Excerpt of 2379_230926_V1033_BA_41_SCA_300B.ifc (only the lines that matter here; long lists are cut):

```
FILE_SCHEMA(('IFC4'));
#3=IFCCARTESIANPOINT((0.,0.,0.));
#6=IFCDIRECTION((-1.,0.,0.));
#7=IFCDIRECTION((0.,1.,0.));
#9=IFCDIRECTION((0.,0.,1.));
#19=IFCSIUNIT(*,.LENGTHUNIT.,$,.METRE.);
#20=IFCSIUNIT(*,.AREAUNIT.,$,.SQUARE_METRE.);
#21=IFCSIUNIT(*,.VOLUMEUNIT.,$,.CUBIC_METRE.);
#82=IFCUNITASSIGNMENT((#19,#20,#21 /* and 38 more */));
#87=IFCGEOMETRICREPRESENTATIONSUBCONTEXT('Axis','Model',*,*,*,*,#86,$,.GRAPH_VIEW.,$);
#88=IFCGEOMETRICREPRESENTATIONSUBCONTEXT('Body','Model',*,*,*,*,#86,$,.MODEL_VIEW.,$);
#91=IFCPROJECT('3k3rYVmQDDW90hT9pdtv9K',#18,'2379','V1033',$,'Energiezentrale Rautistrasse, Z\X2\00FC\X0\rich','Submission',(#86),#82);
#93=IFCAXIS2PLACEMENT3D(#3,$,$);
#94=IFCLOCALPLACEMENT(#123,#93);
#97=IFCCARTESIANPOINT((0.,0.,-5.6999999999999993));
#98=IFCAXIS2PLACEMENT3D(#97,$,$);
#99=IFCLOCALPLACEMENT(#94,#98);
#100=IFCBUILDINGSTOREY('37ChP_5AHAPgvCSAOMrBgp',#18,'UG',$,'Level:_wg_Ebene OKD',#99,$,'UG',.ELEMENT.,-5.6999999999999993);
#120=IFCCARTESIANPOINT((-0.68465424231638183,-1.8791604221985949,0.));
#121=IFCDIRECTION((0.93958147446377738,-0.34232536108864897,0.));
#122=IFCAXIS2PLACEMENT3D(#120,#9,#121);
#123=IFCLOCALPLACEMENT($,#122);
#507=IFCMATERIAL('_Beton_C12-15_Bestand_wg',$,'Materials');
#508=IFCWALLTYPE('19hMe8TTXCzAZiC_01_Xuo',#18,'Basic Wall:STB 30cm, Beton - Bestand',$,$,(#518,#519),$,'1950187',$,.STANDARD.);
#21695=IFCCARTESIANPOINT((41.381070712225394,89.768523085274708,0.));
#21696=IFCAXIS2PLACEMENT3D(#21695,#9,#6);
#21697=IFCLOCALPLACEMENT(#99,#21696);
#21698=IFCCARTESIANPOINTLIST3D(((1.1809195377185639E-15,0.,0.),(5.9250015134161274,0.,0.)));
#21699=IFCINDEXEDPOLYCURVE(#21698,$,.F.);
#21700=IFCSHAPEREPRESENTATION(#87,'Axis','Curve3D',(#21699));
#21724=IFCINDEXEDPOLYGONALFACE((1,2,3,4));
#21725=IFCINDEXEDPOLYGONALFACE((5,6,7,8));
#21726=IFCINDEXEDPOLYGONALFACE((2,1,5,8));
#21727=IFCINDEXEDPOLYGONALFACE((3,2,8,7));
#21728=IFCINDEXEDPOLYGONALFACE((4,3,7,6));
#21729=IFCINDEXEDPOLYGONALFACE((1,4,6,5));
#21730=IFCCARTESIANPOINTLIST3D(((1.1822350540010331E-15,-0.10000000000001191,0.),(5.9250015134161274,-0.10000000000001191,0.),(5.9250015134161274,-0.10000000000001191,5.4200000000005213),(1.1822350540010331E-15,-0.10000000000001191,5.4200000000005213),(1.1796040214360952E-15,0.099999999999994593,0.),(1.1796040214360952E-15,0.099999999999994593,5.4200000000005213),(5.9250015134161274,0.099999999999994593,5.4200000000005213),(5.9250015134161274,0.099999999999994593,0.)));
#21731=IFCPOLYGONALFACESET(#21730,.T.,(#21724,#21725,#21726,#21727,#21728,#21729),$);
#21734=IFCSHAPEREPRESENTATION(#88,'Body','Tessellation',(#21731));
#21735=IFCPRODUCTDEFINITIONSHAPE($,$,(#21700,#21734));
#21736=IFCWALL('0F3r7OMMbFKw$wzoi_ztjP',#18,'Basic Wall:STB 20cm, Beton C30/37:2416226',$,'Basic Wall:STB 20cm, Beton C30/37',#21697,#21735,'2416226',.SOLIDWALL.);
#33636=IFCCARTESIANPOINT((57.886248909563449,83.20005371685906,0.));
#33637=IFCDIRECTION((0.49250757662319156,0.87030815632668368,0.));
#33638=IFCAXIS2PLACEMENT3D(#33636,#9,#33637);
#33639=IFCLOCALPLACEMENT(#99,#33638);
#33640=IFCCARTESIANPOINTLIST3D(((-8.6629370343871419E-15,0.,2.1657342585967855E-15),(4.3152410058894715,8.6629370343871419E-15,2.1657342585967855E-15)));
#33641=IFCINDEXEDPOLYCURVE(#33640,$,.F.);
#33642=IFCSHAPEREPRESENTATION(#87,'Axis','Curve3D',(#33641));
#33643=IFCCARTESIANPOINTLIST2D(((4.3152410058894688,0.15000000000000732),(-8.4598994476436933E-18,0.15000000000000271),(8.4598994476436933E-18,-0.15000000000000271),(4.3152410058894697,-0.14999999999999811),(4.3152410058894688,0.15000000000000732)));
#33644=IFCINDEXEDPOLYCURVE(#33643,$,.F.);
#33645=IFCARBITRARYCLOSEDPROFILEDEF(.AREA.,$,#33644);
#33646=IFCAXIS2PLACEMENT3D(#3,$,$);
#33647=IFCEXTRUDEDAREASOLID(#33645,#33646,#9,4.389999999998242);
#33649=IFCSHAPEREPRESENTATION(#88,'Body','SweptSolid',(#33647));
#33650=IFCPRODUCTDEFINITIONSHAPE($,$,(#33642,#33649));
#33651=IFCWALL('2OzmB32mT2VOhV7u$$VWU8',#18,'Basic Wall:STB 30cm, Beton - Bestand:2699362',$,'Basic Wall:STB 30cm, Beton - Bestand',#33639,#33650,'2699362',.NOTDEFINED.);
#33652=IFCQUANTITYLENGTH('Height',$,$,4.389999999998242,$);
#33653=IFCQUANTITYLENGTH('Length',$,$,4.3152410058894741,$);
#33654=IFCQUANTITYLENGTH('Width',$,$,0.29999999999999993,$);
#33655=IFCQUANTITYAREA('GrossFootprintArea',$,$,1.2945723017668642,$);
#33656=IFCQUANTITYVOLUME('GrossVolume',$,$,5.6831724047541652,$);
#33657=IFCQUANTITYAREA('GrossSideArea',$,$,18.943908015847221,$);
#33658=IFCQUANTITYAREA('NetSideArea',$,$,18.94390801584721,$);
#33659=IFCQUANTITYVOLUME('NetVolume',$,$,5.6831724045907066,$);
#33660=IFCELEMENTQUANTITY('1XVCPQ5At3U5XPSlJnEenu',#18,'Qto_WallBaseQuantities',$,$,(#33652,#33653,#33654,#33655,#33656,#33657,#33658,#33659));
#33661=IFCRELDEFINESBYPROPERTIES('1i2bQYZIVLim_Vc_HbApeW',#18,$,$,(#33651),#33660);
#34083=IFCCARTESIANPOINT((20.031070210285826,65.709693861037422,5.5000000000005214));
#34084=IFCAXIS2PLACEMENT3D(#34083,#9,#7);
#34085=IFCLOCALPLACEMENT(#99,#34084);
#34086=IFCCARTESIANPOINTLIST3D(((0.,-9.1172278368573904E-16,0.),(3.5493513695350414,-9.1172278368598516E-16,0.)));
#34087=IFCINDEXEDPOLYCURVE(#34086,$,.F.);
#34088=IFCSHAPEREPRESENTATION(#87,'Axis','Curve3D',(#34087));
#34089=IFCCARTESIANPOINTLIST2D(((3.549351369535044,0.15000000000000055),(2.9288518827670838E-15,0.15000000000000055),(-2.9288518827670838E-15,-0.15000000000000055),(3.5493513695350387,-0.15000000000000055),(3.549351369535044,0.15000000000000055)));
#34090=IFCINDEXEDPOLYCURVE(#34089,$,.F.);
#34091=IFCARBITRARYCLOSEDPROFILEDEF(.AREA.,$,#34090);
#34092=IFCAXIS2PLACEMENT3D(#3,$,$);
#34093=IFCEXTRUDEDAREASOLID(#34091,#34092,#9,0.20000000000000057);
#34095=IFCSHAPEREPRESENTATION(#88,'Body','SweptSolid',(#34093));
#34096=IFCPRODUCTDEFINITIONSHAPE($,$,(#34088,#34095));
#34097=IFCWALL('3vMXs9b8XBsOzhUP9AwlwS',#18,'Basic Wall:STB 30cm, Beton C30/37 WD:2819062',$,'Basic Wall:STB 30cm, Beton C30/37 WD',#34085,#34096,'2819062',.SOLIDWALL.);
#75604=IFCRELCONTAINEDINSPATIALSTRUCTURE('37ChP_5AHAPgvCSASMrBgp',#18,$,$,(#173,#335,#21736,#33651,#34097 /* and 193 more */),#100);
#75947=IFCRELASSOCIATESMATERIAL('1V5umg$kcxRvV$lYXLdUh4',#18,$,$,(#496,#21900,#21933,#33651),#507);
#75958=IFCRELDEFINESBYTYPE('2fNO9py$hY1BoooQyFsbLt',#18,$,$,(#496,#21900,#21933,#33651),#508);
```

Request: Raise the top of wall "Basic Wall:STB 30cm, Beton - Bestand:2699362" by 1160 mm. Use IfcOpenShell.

```python
import ifcopenshell
import ifcopenshell.api.pset
import ifcopenshell.geom
import ifcopenshell.util.element
import ifcopenshell.util.representation
import ifcopenshell.util.shape
import ifcopenshell.util.unit

model = ifcopenshell.open("2379_230926_V1033_BA_41_SCA_300B.ifc")
unit_scale = ifcopenshell.util.unit.calculate_unit_scale(model)
area_scale = ifcopenshell.util.unit.calculate_unit_scale(model, "AREAUNIT")
volume_scale = ifcopenshell.util.unit.calculate_unit_scale(model, "VOLUMEUNIT")
settings = ifcopenshell.geom.settings()


def volume(element):
    """Net volume in cubic metres, openings subtracted."""
    shape = ifcopenshell.geom.create_shape(settings, element)
    return ifcopenshell.util.shape.get_volume(shape.geometry)


wall = model.by_id(33651)
before = volume(wall)

body = ifcopenshell.util.representation.get_representation(wall, "Model", "Body")
solid = body.Items[0]
old_height = solid.Depth
solid.Depth += 1.16
after = volume(wall)
thickness = 0.3  # wall thickness in metres

# Update the stored height, areas and volumes.
qto = model.by_id(ifcopenshell.util.element.get_pset(wall, "Qto_WallBaseQuantities", should_inherit=False)["id"])
ifcopenshell.api.pset.edit_qto(model, qto=qto, properties={
    "Height": solid.Depth,
    "GrossVolume": ifcopenshell.util.element.get_pset(wall, "Qto_WallBaseQuantities", "GrossVolume") * solid.Depth / old_height,
    "GrossSideArea": ifcopenshell.util.element.get_pset(wall, "Qto_WallBaseQuantities", "GrossSideArea") * solid.Depth / old_height,
    "NetSideArea": after / thickness / area_scale,
    "NetVolume": after / volume_scale,
})

print(f"height {old_height:g} -> {solid.Depth:g}, volume {before:.3f} -> {after:.3f} m3")

model.write("2379_230926_V1033_BA_41_SCA_300B_edited.ifc")
```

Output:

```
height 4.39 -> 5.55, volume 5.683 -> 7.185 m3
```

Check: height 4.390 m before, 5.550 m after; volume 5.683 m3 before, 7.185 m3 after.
